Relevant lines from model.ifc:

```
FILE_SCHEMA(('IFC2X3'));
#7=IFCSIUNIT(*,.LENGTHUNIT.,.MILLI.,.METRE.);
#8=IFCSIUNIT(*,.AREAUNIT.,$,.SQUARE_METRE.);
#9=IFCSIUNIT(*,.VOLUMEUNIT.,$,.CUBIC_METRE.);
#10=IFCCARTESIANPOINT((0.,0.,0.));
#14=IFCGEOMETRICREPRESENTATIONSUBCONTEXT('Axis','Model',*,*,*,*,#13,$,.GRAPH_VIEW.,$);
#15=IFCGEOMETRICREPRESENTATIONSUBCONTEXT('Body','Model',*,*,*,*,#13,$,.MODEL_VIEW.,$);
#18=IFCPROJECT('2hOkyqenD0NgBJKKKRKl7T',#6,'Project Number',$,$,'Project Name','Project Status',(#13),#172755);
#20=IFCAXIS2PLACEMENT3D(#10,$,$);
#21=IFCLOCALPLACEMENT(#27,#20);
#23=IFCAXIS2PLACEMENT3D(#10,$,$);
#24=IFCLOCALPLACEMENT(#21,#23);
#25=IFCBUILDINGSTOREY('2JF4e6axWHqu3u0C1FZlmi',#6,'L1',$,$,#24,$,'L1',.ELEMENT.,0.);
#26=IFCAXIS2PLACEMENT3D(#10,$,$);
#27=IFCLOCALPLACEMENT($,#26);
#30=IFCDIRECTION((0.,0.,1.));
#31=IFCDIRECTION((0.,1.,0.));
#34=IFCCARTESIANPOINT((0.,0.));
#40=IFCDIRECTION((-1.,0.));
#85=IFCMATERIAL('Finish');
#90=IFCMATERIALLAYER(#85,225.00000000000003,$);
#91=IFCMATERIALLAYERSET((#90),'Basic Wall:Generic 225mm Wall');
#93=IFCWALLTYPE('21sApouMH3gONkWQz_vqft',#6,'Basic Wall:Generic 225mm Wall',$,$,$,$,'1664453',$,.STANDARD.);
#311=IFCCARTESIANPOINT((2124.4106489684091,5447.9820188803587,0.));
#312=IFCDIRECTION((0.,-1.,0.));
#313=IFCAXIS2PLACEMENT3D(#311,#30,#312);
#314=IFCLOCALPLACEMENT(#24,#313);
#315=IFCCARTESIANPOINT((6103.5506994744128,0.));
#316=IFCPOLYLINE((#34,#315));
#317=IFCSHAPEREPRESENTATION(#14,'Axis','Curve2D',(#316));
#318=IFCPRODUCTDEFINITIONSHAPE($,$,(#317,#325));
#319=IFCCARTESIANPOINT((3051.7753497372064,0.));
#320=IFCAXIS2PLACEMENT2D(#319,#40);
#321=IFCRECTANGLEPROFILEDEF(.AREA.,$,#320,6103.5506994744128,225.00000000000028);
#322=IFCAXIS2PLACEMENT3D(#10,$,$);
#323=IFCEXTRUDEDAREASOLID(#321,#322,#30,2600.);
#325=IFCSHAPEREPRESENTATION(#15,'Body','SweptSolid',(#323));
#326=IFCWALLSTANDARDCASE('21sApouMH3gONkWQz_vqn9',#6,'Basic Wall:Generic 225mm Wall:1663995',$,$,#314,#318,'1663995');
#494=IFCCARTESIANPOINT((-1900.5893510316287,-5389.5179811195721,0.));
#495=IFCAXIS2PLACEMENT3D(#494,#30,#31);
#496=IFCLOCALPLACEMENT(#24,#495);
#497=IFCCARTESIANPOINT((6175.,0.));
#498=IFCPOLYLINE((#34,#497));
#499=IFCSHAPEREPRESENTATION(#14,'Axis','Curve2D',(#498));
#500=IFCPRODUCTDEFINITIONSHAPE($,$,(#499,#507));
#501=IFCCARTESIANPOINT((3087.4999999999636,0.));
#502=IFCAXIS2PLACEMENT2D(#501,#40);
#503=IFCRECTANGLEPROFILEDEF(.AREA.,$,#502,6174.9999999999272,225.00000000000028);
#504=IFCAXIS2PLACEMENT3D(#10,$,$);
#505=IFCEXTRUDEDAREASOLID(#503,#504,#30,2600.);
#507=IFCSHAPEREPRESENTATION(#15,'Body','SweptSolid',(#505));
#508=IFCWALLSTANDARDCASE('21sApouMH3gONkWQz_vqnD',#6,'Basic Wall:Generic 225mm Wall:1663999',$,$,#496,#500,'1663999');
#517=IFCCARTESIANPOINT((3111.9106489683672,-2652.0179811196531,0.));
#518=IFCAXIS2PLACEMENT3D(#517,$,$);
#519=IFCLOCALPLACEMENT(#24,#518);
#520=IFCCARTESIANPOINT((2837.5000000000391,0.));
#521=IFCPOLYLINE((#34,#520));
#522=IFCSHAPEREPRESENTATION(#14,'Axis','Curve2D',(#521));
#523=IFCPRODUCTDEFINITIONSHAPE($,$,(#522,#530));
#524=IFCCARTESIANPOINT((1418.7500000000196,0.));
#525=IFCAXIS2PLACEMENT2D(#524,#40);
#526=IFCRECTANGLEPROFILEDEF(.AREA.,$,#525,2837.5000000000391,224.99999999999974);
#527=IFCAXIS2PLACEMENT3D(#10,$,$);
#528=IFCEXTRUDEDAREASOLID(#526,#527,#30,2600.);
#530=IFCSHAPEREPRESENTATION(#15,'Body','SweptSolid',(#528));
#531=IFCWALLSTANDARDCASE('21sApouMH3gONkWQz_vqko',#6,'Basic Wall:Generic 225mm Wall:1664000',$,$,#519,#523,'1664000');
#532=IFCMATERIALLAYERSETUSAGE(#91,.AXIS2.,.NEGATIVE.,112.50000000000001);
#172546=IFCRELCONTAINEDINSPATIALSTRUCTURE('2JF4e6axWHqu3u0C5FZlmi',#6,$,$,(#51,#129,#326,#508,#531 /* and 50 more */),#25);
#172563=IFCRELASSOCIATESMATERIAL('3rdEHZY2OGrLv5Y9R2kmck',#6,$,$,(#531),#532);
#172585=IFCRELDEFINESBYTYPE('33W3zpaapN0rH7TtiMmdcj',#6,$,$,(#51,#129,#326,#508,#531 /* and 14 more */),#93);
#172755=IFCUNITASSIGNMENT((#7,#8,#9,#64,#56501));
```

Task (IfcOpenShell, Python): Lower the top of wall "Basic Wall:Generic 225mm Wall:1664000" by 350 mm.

```python
import ifcopenshell
import ifcopenshell.geom
import ifcopenshell.util.representation
import ifcopenshell.util.shape

model = ifcopenshell.open("model.ifc")
settings = ifcopenshell.geom.settings()


def volume(element):
    """Net volume in cubic metres, openings subtracted."""
    shape = ifcopenshell.geom.create_shape(settings, element)
    return ifcopenshell.util.shape.get_volume(shape.geometry)


wall = model.by_guid("21sApouMH3gONkWQz_vqko")
before = volume(wall)

body = ifcopenshell.util.representation.get_representation(wall, "Model", "Body")
solid = body.Items[0]
old_height = solid.Depth
solid.Depth -= 350.0
after = volume(wall)

print(f"height {old_height:g} -> {solid.Depth:g}, volume {before:.3f} -> {after:.3f} m3")

model.write("model_v2.ifc")
```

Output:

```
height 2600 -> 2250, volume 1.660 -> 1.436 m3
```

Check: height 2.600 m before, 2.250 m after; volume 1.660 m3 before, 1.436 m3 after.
